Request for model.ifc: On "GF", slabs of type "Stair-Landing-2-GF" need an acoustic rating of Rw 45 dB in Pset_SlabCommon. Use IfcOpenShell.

First a look at what the model holds.

```python
import ifcopenshell
import ifcopenshell.util.element

model = ifcopenshell.open("model.ifc")
print(model.schema)
storey = next(s for s in model.by_type("IfcBuildingStorey") if s.Name == "GF")
slabs = [e for e in ifcopenshell.util.element.get_decomposition(storey) if e.is_a("IfcSlab")]
seen = {}
for e in slabs:
    element_type = ifcopenshell.util.element.get_type(e)
    key = (element_type.Name if element_type != e and element_type else None, ifcopenshell.util.element.get_pset(e, "Pset_SlabCommon", "AcousticRating"))
    seen[key] = seen.get(key, 0) + 1
for (name, value), count in sorted(seen.items(), key=str):
    print(count, "x", name, "|", value)
```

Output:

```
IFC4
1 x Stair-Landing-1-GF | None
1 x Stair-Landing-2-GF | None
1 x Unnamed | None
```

```python
import ifcopenshell
import ifcopenshell.api.pset
import ifcopenshell.util.element

model = ifcopenshell.open("model.ifc")

storey = next(s for s in model.by_type("IfcBuildingStorey") if s.Name == "GF")
slabs = [e for e in ifcopenshell.util.element.get_decomposition(storey) if e.is_a("IfcSlab")]

count = 0
for e in slabs:
    element_type = ifcopenshell.util.element.get_type(e)
    if element_type in (None, e) or element_type.Name != "Stair-Landing-2-GF":
        continue
    # add_pset returns the element's existing set when there is one.
    pset = ifcopenshell.api.pset.add_pset(model, product=e, name="Pset_SlabCommon")
    ifcopenshell.api.pset.edit_pset(model, pset=pset, properties={"AcousticRating": "Rw 45 dB"})
    count += 1

print(count, "slabs updated")

model.write("model_edited.ifc")
```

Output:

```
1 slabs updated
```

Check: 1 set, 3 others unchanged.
